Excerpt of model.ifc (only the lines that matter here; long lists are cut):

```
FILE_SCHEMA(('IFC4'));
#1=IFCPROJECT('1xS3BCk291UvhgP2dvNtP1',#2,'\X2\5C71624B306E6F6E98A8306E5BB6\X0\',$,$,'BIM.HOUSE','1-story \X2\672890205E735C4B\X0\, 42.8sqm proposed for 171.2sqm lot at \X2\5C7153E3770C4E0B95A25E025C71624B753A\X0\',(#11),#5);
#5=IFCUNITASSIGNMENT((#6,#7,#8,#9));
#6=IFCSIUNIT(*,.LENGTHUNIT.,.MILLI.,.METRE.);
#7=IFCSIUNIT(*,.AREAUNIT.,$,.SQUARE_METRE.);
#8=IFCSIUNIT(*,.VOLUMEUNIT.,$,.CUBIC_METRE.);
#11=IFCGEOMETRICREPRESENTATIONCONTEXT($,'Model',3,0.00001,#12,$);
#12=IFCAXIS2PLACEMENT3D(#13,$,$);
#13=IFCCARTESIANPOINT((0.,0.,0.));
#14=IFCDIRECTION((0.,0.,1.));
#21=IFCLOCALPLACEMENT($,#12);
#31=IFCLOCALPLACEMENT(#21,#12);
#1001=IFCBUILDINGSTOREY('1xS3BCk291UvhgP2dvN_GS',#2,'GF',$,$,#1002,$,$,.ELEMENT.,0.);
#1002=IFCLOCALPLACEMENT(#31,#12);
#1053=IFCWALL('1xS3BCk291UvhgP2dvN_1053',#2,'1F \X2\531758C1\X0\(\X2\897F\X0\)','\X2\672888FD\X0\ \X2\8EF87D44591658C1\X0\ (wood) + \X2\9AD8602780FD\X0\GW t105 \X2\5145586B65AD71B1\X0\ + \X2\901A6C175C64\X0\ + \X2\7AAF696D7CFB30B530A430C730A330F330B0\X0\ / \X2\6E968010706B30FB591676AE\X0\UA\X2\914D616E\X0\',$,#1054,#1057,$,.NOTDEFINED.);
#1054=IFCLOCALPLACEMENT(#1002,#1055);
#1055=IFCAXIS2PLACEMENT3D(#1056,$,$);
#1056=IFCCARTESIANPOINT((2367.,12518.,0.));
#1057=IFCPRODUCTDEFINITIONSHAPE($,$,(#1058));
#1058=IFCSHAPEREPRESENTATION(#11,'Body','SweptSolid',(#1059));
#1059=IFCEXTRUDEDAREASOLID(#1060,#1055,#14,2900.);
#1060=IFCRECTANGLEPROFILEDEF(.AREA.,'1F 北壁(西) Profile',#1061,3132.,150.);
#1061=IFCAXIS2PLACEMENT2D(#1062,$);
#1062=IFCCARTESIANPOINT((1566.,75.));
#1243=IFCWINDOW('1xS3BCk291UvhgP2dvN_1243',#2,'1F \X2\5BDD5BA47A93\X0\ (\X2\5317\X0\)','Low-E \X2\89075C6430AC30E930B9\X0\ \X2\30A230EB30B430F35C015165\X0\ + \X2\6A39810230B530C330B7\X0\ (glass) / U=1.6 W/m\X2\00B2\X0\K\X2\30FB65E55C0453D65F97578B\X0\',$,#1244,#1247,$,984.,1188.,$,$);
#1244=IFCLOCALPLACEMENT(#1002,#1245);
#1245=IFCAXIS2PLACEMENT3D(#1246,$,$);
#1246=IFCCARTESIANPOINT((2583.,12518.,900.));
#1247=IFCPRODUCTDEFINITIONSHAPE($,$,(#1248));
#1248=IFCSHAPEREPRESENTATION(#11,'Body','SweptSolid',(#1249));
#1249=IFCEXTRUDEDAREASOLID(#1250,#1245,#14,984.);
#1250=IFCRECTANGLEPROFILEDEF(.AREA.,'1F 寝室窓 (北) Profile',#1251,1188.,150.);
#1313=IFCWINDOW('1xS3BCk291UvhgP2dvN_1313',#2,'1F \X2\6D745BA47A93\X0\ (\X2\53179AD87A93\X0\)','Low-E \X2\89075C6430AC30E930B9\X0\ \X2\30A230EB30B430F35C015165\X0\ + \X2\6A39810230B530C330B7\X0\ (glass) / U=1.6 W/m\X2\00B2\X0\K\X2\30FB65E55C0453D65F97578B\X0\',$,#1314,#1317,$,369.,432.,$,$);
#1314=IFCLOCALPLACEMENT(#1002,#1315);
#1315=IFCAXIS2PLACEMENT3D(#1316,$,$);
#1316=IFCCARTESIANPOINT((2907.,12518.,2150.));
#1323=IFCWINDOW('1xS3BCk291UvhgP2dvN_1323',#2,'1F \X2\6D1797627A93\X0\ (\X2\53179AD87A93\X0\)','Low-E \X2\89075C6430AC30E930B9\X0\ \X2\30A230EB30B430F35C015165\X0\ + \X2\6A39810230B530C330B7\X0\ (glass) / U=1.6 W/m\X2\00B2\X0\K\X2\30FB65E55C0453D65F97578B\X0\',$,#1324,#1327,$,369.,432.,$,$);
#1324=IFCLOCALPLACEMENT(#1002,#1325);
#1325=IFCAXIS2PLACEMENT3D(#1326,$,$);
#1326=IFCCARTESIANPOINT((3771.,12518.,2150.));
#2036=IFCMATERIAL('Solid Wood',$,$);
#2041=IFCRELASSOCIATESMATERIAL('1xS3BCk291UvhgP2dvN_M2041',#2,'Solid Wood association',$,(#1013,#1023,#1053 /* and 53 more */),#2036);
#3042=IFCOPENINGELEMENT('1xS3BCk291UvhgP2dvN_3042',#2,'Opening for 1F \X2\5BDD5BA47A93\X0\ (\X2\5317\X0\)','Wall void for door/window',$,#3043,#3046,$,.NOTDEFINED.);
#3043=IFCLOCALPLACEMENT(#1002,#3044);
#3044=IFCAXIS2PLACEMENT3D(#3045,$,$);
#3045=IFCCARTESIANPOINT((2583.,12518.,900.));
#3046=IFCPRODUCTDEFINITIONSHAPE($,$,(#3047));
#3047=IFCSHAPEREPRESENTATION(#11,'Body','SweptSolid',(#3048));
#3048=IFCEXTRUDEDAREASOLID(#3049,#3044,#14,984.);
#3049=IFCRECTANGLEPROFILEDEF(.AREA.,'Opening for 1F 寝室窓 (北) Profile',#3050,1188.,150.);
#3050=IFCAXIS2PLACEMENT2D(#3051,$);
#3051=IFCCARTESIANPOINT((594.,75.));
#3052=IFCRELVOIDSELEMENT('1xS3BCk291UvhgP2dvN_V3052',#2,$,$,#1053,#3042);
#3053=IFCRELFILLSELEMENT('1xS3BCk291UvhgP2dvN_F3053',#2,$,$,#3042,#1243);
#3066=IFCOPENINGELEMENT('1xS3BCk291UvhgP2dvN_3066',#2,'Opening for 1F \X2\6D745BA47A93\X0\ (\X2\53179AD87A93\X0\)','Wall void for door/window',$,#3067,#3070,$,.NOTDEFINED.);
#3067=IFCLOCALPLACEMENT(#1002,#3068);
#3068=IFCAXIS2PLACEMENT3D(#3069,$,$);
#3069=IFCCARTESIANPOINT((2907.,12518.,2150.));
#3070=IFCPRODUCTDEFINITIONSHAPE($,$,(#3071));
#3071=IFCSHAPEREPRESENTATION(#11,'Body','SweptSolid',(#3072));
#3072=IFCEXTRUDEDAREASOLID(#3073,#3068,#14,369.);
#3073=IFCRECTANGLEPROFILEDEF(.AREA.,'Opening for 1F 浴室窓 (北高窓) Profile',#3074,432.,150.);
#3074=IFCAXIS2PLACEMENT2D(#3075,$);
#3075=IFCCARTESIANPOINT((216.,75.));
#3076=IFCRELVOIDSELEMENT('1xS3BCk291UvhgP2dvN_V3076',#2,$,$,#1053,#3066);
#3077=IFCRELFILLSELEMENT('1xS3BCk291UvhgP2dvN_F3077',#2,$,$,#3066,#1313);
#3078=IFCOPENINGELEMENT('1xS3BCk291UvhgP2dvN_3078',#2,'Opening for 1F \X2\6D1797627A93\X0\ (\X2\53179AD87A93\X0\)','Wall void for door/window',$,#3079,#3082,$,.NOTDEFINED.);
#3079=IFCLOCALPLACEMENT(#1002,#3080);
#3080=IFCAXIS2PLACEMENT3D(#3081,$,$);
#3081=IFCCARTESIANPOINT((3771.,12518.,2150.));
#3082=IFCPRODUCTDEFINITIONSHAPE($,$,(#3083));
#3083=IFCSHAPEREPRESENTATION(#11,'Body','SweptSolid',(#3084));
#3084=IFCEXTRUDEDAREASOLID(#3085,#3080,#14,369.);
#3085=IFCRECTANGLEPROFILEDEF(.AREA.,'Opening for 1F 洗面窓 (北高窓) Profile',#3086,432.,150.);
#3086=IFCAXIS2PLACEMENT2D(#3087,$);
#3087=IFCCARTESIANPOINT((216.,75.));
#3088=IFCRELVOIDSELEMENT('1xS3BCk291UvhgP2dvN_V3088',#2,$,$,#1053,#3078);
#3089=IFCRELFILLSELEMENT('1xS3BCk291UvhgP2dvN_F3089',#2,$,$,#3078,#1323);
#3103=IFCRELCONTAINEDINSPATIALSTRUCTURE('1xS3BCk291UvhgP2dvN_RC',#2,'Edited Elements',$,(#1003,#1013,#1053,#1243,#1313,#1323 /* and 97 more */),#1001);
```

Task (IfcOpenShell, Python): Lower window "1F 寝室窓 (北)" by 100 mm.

```python
import numpy as np
import ifcopenshell
import ifcopenshell.api.geometry
import ifcopenshell.util.placement
import ifcopenshell.util.unit

model = ifcopenshell.open("model.ifc")
unit_scale = ifcopenshell.util.unit.calculate_unit_scale(model)

window = model.by_guid("1xS3BCk291UvhgP2dvN_1243")
opening = window.FillsVoids[0].RelatingOpeningElement
dz = -100.0

shift = np.array([0.0, 0.0, dz])
# The window is not placed relative to its opening, so move both.
for product in (opening, window):
    matrix = ifcopenshell.util.placement.get_local_placement(product.ObjectPlacement)
    matrix[:3, 3] += shift
    ifcopenshell.api.geometry.edit_object_placement(model, product=product, matrix=matrix, is_si=False)

print(f"moved by {dz * unit_scale:+.3f} m")

model.write("model-out.ifc")
```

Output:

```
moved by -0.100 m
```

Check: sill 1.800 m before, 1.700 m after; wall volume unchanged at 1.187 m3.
